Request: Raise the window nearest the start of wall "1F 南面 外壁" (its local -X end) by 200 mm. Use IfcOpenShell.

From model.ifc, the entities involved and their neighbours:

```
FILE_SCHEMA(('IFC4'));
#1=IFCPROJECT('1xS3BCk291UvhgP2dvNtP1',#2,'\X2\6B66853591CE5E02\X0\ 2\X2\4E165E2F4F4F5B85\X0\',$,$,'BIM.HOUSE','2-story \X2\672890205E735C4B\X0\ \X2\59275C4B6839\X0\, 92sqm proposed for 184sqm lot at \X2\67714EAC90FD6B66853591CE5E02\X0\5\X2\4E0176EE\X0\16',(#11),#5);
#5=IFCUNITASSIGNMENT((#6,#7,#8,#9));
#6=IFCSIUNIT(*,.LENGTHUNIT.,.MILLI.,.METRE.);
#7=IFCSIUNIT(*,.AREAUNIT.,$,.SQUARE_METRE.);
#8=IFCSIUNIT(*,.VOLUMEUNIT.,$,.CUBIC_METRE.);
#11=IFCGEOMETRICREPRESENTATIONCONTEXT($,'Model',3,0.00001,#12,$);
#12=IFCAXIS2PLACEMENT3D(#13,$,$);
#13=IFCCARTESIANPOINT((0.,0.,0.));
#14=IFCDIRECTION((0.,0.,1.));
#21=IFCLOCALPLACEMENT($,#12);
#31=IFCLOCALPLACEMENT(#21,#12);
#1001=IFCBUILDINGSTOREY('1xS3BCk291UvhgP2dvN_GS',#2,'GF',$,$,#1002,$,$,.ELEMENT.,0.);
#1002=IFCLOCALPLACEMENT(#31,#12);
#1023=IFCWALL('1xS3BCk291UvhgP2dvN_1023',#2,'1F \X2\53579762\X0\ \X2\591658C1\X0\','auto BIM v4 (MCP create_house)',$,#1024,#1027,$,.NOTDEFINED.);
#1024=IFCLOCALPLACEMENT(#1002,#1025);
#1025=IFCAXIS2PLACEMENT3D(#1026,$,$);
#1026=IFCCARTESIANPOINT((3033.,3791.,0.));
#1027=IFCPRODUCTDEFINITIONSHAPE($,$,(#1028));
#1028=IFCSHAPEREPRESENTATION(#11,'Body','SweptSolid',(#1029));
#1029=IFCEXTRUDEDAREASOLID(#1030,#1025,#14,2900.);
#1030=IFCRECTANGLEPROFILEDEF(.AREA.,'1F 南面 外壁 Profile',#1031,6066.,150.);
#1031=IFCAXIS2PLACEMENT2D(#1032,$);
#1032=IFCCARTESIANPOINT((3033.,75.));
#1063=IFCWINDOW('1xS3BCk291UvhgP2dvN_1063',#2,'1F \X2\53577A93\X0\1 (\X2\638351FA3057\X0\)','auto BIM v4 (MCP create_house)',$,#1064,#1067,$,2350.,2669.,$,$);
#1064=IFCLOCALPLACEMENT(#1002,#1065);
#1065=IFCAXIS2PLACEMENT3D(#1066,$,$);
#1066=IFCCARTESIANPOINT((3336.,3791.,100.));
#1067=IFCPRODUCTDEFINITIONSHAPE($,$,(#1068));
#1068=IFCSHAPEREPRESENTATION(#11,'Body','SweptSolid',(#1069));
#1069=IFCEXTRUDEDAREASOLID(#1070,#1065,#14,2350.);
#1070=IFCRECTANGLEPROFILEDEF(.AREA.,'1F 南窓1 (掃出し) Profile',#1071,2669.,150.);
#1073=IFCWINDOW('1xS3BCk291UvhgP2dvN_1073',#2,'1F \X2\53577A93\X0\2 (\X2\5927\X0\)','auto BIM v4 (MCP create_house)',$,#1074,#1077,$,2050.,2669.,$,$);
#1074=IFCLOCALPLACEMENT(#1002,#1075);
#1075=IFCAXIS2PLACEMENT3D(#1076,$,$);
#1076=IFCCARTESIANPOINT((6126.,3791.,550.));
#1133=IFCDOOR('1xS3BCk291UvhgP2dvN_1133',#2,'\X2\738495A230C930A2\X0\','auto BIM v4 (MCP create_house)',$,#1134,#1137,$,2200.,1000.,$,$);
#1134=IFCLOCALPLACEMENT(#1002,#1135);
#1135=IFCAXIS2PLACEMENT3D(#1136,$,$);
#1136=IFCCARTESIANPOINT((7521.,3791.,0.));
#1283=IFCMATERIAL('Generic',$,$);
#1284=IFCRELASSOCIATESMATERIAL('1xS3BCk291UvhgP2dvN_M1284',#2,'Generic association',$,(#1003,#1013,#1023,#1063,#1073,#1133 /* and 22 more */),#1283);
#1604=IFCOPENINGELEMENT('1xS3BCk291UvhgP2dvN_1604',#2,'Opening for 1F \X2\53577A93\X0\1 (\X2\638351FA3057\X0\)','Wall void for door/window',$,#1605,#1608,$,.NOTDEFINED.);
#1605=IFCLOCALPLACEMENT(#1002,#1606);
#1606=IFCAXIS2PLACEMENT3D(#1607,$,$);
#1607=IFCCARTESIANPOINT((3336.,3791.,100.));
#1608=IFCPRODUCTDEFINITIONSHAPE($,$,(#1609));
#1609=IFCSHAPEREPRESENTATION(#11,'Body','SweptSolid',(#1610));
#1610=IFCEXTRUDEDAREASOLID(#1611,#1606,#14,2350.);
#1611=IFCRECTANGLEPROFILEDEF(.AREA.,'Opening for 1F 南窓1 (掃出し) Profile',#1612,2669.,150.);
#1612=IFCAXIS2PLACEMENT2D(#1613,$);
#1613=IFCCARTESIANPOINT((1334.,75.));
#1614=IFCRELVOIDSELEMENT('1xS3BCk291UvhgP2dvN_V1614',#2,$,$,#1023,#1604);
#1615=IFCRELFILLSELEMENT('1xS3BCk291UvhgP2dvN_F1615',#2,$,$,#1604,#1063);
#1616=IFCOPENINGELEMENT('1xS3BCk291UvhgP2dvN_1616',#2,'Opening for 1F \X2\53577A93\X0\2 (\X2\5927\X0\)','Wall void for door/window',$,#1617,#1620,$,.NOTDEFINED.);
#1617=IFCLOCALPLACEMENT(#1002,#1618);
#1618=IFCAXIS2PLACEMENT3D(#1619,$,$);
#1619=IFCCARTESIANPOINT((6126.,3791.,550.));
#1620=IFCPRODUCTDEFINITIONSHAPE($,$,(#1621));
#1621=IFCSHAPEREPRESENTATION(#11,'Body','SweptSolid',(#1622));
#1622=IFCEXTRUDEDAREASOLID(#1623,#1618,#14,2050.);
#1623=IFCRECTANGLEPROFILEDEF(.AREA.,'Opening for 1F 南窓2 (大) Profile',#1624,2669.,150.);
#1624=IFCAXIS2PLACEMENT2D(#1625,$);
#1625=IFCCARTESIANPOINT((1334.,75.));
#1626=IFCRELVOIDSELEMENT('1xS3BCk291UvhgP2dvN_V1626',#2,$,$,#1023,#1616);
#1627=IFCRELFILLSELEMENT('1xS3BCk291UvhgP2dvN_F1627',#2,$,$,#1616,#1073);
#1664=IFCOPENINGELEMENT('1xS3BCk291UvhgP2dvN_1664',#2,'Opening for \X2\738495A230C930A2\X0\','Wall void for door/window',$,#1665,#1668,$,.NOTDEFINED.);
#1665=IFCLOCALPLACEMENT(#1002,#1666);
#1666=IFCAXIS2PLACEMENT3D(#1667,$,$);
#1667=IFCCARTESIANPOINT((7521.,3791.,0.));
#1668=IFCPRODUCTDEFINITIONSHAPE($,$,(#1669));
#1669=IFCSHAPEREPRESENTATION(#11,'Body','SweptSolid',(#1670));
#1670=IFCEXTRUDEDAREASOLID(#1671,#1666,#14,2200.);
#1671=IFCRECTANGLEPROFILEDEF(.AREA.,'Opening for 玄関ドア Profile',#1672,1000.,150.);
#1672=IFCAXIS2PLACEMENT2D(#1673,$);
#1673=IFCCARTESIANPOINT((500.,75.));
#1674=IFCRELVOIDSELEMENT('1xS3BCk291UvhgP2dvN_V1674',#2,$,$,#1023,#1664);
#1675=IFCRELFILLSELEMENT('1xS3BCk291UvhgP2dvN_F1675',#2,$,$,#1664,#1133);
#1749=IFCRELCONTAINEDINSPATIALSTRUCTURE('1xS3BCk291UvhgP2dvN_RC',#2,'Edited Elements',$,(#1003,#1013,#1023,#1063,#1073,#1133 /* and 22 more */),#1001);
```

```python
import numpy as np
import ifcopenshell
import ifcopenshell.api.geometry
import ifcopenshell.util.placement
import ifcopenshell.util.unit

model = ifcopenshell.open("model.ifc")
unit_scale = ifcopenshell.util.unit.calculate_unit_scale(model)

window = model.by_guid("1xS3BCk291UvhgP2dvN_1063")
opening = window.FillsVoids[0].RelatingOpeningElement
dz = 0.2 / unit_scale

shift = np.array([0.0, 0.0, dz])
# The window is not placed relative to its opening, so move both.
for product in (opening, window):
    matrix = ifcopenshell.util.placement.get_local_placement(product.ObjectPlacement)
    matrix[:3, 3] += shift
    ifcopenshell.api.geometry.edit_object_placement(model, product=product, matrix=matrix, is_si=False)

print(f"moved by {dz * unit_scale:+.3f} m")

model.write("model-out.ifc")
```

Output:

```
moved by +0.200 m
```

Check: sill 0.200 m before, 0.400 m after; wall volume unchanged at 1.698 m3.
